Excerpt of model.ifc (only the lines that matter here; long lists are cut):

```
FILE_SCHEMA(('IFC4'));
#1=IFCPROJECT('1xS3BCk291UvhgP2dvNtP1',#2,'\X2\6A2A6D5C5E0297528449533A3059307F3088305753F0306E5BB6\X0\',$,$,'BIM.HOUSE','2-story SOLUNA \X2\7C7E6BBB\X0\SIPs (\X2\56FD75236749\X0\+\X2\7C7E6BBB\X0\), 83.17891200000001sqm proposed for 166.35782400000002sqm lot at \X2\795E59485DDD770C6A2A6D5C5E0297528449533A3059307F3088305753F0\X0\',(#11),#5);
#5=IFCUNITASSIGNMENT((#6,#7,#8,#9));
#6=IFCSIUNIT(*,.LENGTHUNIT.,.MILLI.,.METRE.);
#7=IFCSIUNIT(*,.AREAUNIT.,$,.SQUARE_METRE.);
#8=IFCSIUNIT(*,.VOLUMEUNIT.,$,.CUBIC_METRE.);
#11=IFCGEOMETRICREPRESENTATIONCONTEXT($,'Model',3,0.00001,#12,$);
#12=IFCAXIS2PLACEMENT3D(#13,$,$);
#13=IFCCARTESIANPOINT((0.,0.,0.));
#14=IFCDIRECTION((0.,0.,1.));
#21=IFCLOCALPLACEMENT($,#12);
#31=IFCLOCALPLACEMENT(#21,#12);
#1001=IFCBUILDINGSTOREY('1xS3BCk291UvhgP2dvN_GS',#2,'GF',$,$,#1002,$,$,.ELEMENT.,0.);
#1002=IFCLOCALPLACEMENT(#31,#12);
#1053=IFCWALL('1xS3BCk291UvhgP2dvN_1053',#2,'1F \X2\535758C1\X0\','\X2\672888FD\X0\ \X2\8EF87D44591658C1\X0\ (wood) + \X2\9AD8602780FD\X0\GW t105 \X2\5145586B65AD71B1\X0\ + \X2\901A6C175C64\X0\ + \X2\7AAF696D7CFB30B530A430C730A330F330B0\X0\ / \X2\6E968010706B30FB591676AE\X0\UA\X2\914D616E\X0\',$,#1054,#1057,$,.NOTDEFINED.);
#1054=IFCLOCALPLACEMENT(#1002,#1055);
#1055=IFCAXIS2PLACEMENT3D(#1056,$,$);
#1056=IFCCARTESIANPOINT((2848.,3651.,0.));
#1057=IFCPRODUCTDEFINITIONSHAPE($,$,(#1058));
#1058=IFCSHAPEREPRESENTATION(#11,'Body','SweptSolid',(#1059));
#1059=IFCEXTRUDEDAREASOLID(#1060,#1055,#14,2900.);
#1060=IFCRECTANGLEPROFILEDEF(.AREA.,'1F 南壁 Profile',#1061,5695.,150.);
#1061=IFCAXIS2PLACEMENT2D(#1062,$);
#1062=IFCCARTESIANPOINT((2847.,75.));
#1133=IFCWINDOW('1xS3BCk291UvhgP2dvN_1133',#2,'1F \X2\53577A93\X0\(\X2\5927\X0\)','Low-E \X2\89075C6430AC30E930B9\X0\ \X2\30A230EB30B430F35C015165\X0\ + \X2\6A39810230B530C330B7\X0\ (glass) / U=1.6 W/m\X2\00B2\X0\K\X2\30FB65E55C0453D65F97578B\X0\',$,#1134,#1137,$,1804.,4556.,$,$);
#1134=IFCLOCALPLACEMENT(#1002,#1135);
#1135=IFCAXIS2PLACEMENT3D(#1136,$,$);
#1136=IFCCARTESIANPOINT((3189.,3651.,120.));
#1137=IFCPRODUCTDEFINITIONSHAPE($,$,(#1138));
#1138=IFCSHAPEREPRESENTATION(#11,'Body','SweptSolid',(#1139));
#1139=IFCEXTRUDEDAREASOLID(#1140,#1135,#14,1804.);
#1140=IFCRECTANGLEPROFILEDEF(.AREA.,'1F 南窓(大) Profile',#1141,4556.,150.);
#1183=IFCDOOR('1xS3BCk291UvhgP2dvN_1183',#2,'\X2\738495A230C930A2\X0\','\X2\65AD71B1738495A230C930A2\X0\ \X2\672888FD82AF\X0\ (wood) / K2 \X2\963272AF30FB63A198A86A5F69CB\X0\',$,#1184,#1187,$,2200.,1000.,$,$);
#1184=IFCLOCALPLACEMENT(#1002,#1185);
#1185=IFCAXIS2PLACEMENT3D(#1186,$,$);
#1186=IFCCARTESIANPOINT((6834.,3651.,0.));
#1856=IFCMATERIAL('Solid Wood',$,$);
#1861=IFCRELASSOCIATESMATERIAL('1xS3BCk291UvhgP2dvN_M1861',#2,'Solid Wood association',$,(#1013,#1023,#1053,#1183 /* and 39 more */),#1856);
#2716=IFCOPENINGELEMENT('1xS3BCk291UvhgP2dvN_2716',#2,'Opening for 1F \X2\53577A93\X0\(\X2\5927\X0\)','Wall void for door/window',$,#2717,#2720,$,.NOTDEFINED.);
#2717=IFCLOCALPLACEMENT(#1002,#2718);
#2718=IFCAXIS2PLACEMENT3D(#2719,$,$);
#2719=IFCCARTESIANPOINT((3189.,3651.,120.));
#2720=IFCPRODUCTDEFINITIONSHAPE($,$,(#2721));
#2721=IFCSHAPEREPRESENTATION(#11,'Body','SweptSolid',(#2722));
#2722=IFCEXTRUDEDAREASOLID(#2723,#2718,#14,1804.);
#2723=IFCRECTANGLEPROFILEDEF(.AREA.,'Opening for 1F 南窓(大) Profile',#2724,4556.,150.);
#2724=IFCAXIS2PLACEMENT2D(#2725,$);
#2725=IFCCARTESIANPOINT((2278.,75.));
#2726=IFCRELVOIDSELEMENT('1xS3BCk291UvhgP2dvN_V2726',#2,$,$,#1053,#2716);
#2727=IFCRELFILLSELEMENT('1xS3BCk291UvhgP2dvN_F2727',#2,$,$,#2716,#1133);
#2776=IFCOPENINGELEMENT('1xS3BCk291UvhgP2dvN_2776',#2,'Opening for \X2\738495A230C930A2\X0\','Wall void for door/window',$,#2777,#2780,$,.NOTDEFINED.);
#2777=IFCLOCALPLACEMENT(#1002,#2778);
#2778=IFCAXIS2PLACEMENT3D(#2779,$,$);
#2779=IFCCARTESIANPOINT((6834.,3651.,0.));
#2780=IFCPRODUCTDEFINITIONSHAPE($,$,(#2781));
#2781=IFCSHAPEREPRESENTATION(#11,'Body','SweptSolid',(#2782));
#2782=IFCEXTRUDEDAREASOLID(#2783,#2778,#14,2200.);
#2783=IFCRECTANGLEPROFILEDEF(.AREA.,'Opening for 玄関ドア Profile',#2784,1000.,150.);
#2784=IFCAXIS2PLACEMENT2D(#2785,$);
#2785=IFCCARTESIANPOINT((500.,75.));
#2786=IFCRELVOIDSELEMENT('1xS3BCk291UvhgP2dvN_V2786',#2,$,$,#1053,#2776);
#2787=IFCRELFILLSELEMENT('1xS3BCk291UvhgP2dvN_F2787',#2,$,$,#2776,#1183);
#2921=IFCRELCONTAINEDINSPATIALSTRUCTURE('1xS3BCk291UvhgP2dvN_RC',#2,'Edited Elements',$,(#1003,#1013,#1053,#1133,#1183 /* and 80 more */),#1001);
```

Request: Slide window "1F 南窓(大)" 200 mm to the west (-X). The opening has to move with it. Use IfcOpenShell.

```python
import ifcopenshell
import ifcopenshell.api.geometry
import ifcopenshell.util.placement
import ifcopenshell.util.unit

model = ifcopenshell.open("model.ifc")
unit_scale = ifcopenshell.util.unit.calculate_unit_scale(model)

window = model.by_guid("1xS3BCk291UvhgP2dvN_1133")
opening = window.FillsVoids[0].RelatingOpeningElement
wall = opening.VoidsElements[0].RelatingBuildingElement

wall_matrix = ifcopenshell.util.placement.get_local_placement(wall.ObjectPlacement)
shift = wall_matrix[:3, 0] * -0.2 / unit_scale
before = ifcopenshell.util.placement.get_local_placement(window.ObjectPlacement)[:3, 3].copy()

# The window is not placed relative to its opening, so move both.
for product in (opening, window):
    matrix = ifcopenshell.util.placement.get_local_placement(product.ObjectPlacement)
    matrix[:3, 3] += shift
    ifcopenshell.api.geometry.edit_object_placement(model, product=product, matrix=matrix, is_si=False)

after = ifcopenshell.util.placement.get_local_placement(window.ObjectPlacement)[:3, 3]
print("window moved by", (after - before).round(3) + 0.0)

model.write("model_rev.ifc")
```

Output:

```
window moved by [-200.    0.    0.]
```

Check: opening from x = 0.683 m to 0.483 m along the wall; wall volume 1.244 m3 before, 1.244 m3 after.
